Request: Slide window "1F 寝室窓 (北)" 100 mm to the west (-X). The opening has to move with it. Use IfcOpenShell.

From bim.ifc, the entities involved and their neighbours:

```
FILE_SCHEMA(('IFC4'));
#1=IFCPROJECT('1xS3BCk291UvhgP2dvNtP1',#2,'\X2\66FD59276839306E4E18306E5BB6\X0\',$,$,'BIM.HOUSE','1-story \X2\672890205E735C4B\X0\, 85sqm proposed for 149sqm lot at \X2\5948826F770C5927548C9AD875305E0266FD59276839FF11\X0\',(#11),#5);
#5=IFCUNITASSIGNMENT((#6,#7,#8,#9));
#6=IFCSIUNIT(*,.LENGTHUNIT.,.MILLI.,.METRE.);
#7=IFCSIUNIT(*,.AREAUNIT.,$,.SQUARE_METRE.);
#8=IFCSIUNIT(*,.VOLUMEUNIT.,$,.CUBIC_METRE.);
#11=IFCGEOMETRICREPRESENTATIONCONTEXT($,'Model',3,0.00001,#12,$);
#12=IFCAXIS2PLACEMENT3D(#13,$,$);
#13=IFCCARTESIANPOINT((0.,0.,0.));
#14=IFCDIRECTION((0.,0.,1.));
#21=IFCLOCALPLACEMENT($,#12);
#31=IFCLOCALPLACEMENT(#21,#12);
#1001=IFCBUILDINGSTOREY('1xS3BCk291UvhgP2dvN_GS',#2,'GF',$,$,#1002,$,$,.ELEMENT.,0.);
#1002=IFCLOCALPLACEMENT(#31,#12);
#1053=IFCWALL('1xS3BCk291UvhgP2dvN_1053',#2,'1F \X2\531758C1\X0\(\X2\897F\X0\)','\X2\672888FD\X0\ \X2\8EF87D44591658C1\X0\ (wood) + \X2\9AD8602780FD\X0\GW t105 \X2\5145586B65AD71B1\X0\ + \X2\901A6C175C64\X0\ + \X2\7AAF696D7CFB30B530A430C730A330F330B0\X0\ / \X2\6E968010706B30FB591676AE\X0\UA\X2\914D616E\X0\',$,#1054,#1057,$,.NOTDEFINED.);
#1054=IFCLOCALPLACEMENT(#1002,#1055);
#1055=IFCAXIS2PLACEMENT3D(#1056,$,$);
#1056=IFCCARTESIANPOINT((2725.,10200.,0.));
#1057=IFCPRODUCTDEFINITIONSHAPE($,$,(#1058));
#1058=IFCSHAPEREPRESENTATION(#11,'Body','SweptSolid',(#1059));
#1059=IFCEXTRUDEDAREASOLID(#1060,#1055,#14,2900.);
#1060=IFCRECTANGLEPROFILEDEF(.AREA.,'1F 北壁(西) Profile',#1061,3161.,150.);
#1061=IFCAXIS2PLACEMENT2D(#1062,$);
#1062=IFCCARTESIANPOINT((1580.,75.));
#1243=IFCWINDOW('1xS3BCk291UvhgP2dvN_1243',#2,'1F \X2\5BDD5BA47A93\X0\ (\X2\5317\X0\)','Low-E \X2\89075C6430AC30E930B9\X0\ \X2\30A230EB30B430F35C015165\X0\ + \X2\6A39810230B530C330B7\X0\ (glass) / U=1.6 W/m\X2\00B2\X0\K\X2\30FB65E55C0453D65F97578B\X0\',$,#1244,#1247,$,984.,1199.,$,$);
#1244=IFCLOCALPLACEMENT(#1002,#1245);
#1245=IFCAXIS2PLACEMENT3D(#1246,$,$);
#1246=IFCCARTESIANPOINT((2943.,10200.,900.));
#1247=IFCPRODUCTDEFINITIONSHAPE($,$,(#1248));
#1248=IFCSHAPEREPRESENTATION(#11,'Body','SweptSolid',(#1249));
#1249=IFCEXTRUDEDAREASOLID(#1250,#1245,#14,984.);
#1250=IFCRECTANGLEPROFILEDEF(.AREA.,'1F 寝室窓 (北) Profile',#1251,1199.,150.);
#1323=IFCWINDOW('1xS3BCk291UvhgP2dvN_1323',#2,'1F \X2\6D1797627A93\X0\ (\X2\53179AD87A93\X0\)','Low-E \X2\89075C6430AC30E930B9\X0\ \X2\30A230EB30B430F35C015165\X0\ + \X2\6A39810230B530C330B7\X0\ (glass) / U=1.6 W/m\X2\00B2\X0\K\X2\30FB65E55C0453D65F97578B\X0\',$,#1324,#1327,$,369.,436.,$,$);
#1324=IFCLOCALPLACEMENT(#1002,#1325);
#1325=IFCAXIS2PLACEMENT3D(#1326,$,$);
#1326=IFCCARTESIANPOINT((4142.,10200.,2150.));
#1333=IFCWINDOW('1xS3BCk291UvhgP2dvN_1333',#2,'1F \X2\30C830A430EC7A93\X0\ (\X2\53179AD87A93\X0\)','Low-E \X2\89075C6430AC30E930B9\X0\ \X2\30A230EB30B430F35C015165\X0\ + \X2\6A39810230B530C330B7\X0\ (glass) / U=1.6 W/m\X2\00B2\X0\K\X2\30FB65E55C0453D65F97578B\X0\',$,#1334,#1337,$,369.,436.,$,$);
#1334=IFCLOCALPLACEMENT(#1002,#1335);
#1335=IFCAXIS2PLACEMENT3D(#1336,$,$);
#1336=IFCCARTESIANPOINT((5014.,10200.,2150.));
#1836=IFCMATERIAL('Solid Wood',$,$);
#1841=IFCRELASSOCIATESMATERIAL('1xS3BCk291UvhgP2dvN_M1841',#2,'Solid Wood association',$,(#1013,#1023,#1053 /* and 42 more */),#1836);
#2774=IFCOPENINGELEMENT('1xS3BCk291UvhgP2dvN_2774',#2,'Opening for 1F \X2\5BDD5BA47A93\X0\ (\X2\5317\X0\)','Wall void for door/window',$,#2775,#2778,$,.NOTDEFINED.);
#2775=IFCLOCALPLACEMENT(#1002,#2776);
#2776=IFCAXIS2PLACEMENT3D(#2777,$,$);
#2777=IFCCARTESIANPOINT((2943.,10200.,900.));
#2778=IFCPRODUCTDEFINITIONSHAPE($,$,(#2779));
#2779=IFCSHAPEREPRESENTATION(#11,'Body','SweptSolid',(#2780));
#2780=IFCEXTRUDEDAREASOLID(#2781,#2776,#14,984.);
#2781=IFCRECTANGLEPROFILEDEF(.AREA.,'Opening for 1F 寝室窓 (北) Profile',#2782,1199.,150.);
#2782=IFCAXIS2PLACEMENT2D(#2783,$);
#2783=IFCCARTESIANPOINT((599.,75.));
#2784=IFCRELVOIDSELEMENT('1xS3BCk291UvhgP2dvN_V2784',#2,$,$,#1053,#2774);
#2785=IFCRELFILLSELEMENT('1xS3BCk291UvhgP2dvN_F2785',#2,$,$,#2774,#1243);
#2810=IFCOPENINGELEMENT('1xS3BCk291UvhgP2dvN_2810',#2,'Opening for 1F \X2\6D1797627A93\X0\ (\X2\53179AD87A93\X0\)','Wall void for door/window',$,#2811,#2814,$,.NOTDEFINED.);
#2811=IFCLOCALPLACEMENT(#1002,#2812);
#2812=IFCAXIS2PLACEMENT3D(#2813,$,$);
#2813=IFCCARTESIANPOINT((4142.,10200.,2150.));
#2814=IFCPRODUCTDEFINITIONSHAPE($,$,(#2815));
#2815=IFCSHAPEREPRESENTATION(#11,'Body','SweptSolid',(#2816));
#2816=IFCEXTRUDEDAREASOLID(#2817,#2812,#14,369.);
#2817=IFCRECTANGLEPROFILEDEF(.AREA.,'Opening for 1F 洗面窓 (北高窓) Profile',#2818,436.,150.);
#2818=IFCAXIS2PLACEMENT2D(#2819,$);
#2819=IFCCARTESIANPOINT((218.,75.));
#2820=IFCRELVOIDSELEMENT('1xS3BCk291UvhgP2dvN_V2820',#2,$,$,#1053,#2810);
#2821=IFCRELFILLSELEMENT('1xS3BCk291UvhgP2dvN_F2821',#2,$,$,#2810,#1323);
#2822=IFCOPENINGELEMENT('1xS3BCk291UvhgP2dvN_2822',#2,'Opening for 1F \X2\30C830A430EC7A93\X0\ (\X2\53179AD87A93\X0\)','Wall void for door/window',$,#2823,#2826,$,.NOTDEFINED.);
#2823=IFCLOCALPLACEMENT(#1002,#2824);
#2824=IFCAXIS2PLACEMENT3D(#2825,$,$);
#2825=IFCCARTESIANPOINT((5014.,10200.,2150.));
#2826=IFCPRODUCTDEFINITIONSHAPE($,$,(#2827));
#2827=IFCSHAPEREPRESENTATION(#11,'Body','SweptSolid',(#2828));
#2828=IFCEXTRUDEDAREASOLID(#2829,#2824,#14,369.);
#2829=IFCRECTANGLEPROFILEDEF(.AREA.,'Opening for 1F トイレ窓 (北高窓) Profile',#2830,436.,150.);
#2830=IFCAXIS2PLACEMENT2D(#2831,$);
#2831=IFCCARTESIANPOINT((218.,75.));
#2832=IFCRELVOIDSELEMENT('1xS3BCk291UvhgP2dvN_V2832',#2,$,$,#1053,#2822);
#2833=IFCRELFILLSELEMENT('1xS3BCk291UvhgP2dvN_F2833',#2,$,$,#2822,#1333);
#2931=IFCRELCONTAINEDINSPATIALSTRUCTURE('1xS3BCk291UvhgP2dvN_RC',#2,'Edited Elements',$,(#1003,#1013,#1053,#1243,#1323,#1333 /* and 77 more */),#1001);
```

```python
import ifcopenshell
import ifcopenshell.api.geometry
import ifcopenshell.util.placement
import ifcopenshell.util.unit

model = ifcopenshell.open("bim.ifc")
unit_scale = ifcopenshell.util.unit.calculate_unit_scale(model)

window = model.by_id(1243)
opening = window.FillsVoids[0].RelatingOpeningElement
wall = opening.VoidsElements[0].RelatingBuildingElement

wall_matrix = ifcopenshell.util.placement.get_local_placement(wall.ObjectPlacement)
shift = wall_matrix[:3, 0] * -0.1 / unit_scale
before = ifcopenshell.util.placement.get_local_placement(window.ObjectPlacement)[:3, 3].copy()

# The window is not placed relative to its opening, so move both.
for product in (opening, window):
    matrix = ifcopenshell.util.placement.get_local_placement(product.ObjectPlacement)
    matrix[:3, 3] += shift
    ifcopenshell.api.geometry.edit_object_placement(model, product=product, matrix=matrix, is_si=False)

after = ifcopenshell.util.placement.get_local_placement(window.ObjectPlacement)[:3, 3]
print("window moved by", (after - before).round(3) + 0.0)

model.write("bim_updated.ifc")
```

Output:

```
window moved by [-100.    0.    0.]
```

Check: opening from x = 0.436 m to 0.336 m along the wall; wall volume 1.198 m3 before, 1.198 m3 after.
